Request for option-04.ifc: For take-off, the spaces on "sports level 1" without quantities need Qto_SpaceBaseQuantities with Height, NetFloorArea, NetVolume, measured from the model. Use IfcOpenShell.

First a look at what the model holds.

```python
import ifcopenshell
import ifcopenshell.util.element
import ifcopenshell.util.unit

model = ifcopenshell.open("option-04.ifc")
print(model.schema)
for unit_type in ("LENGTHUNIT", "AREAUNIT", "VOLUMEUNIT"):
    print(unit_type, ifcopenshell.util.unit.calculate_unit_scale(model, unit_type))
storey = next(s for s in model.by_type("IfcBuildingStorey") if s.Name == "sports level 1")
spaces = [e for e in ifcopenshell.util.element.get_decomposition(storey) if e.is_a("IfcSpace")]
for e in sorted(spaces, key=lambda e: e.id()):
    print(e.id(), e.is_a(), e.Name, list(ifcopenshell.util.element.get_psets(e, qtos_only=True)), sep=" | ")
```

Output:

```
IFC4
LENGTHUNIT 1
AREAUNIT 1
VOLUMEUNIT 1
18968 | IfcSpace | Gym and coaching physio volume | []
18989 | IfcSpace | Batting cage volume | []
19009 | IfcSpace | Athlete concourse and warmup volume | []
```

```python
import ifcopenshell
import ifcopenshell.api.pset
import ifcopenshell.geom
import ifcopenshell.util.element
import ifcopenshell.util.shape
import ifcopenshell.util.unit

model = ifcopenshell.open("option-04.ifc")
unit_scale = ifcopenshell.util.unit.calculate_unit_scale(model)
area_scale = ifcopenshell.util.unit.calculate_unit_scale(model, "AREAUNIT")
volume_scale = ifcopenshell.util.unit.calculate_unit_scale(model, "VOLUMEUNIT")
settings = ifcopenshell.geom.settings()

storey = next(s for s in model.by_type("IfcBuildingStorey") if s.Name == "sports level 1")
spaces = [e for e in ifcopenshell.util.element.get_decomposition(storey) if e.is_a("IfcSpace")]

for e in sorted(spaces, key=lambda e: e.id()):
    if ifcopenshell.util.element.get_psets(e, qtos_only=True, should_inherit=False):
        continue
    # Geometry comes back in metres, in the element's own axes.
    shape = ifcopenshell.geom.create_shape(settings, e)
    values = {
        "Height": ifcopenshell.util.shape.get_z(shape.geometry) / unit_scale,
        "NetFloorArea": ifcopenshell.util.shape.get_footprint_area(shape.geometry) / area_scale,
        "NetVolume": ifcopenshell.util.shape.get_volume(shape.geometry) / volume_scale,
    }
    qto = ifcopenshell.api.pset.add_qto(model, product=e, name="Qto_SpaceBaseQuantities")
    ifcopenshell.api.pset.edit_qto(model, qto=qto, properties=values)
    print(e.id(), {k: round(v, 3) for k, v in values.items()})

model.write("option-04-out.ifc")
```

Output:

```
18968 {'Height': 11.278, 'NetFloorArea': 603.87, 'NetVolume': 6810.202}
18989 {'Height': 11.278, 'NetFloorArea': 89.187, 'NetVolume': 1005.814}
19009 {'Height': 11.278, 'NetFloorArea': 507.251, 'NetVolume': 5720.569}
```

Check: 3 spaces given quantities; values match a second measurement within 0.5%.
